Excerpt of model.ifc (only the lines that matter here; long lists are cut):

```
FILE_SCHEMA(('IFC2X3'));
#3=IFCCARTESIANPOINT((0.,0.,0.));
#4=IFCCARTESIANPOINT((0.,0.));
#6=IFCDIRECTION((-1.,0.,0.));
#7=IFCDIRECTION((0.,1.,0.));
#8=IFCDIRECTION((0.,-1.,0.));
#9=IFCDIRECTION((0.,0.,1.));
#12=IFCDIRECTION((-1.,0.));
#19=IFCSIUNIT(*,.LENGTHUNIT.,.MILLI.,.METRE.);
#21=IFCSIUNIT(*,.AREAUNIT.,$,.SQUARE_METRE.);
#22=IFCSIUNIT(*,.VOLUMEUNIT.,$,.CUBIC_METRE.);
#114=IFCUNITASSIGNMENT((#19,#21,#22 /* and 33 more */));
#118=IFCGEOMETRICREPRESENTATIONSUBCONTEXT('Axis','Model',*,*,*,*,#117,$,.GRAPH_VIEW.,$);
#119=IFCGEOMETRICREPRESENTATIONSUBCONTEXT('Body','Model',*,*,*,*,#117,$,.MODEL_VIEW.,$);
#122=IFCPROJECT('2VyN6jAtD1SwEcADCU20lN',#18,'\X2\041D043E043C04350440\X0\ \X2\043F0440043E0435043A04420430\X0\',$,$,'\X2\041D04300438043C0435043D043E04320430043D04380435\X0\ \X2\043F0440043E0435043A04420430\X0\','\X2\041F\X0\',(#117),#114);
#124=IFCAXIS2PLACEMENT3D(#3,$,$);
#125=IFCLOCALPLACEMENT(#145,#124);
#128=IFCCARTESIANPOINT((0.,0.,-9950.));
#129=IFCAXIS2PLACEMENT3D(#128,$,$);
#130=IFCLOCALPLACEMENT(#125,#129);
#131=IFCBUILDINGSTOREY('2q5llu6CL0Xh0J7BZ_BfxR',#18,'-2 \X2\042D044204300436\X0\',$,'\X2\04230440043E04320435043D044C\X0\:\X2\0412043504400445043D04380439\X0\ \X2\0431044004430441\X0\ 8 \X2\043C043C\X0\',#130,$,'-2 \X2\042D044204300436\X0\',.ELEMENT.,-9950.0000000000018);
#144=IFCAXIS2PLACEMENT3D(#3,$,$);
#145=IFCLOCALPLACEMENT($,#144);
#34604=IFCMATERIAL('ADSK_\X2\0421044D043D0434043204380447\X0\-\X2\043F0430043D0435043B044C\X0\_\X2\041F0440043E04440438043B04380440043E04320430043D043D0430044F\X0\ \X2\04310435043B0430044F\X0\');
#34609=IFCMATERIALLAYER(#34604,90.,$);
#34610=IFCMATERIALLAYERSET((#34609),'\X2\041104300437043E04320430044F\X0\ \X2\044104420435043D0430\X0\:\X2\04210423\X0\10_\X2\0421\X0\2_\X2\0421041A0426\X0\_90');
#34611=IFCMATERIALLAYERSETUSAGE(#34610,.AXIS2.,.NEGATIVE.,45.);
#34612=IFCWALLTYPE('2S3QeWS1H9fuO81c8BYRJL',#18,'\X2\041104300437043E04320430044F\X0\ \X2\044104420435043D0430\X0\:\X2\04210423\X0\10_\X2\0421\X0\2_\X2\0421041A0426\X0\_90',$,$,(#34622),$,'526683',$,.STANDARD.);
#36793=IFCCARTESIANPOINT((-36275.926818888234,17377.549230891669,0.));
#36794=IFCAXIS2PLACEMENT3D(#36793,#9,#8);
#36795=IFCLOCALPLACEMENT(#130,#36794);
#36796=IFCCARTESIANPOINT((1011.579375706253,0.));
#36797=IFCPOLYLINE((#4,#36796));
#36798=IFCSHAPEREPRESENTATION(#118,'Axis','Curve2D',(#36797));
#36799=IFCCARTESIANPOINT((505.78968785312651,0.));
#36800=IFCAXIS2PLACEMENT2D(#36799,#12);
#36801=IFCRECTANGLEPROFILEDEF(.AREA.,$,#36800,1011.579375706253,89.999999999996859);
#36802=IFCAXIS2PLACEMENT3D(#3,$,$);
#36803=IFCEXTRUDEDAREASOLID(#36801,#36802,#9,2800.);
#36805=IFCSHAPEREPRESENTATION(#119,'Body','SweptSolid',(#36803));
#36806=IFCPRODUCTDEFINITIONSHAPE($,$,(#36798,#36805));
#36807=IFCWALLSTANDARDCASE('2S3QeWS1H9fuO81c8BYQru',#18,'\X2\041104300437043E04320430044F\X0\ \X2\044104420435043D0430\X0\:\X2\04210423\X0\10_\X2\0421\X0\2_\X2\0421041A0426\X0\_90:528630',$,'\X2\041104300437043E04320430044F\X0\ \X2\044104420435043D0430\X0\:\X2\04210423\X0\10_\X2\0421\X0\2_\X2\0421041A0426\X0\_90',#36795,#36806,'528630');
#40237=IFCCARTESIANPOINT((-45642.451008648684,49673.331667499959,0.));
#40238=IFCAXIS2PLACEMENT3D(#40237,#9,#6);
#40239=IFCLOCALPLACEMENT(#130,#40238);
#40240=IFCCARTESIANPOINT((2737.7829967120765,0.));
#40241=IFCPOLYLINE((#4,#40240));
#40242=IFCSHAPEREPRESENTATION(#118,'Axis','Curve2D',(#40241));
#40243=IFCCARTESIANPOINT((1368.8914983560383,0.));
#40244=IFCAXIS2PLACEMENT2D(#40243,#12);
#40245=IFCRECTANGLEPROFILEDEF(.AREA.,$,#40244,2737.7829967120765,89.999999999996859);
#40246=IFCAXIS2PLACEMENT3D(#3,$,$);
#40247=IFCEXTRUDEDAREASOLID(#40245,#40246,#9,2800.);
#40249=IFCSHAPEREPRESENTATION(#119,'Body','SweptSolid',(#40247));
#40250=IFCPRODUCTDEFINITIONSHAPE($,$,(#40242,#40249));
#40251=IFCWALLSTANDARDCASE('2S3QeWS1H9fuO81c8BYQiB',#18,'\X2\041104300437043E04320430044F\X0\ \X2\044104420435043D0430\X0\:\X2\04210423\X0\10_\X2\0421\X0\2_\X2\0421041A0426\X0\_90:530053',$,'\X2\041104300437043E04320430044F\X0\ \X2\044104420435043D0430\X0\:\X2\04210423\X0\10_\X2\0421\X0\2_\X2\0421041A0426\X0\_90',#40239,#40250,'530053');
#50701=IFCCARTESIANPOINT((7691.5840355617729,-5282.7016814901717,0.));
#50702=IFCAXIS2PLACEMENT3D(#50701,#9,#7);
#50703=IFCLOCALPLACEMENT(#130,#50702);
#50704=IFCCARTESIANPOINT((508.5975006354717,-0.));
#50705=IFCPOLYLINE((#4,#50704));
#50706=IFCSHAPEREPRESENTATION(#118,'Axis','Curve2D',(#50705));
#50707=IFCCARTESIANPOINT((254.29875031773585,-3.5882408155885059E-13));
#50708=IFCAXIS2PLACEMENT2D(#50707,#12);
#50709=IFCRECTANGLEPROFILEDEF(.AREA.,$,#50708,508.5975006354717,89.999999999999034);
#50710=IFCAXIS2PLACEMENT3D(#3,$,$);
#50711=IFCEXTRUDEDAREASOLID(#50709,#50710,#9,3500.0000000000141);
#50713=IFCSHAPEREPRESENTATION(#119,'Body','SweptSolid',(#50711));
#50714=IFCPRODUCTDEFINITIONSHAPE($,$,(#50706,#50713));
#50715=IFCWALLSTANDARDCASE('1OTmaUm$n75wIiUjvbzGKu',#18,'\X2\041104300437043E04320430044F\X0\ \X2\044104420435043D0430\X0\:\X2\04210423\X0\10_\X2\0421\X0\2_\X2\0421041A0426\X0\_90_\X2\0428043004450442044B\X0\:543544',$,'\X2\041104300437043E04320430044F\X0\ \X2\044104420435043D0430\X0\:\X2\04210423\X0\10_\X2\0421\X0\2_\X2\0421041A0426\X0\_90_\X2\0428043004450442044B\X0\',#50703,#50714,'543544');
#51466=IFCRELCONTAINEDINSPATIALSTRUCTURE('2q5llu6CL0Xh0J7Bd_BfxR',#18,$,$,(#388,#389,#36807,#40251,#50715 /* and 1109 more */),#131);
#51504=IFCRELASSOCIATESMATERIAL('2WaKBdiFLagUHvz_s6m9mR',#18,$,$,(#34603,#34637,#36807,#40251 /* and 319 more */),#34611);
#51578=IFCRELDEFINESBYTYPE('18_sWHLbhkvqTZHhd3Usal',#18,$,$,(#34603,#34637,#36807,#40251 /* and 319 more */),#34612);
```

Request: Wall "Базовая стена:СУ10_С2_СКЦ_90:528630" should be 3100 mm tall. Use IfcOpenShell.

```python
import ifcopenshell
import ifcopenshell.geom
import ifcopenshell.util.representation
import ifcopenshell.util.shape
import ifcopenshell.util.unit

model = ifcopenshell.open("model.ifc")
unit_scale = ifcopenshell.util.unit.calculate_unit_scale(model)
settings = ifcopenshell.geom.settings()


def volume(element):
    """Net volume in cubic metres, openings subtracted."""
    shape = ifcopenshell.geom.create_shape(settings, element)
    return ifcopenshell.util.shape.get_volume(shape.geometry)


wall = model.by_guid("2S3QeWS1H9fuO81c8BYQru")
before = volume(wall)

body = ifcopenshell.util.representation.get_representation(wall, "Model", "Body")
solid = body.Items[0]
old_height = solid.Depth
solid.Depth = 3.1 / unit_scale
after = volume(wall)

print(f"height {old_height:g} -> {solid.Depth:g}, volume {before:.3f} -> {after:.3f} m3")

model.write("model-out.ifc")
```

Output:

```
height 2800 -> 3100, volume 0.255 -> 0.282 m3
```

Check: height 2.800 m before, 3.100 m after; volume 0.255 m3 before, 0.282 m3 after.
